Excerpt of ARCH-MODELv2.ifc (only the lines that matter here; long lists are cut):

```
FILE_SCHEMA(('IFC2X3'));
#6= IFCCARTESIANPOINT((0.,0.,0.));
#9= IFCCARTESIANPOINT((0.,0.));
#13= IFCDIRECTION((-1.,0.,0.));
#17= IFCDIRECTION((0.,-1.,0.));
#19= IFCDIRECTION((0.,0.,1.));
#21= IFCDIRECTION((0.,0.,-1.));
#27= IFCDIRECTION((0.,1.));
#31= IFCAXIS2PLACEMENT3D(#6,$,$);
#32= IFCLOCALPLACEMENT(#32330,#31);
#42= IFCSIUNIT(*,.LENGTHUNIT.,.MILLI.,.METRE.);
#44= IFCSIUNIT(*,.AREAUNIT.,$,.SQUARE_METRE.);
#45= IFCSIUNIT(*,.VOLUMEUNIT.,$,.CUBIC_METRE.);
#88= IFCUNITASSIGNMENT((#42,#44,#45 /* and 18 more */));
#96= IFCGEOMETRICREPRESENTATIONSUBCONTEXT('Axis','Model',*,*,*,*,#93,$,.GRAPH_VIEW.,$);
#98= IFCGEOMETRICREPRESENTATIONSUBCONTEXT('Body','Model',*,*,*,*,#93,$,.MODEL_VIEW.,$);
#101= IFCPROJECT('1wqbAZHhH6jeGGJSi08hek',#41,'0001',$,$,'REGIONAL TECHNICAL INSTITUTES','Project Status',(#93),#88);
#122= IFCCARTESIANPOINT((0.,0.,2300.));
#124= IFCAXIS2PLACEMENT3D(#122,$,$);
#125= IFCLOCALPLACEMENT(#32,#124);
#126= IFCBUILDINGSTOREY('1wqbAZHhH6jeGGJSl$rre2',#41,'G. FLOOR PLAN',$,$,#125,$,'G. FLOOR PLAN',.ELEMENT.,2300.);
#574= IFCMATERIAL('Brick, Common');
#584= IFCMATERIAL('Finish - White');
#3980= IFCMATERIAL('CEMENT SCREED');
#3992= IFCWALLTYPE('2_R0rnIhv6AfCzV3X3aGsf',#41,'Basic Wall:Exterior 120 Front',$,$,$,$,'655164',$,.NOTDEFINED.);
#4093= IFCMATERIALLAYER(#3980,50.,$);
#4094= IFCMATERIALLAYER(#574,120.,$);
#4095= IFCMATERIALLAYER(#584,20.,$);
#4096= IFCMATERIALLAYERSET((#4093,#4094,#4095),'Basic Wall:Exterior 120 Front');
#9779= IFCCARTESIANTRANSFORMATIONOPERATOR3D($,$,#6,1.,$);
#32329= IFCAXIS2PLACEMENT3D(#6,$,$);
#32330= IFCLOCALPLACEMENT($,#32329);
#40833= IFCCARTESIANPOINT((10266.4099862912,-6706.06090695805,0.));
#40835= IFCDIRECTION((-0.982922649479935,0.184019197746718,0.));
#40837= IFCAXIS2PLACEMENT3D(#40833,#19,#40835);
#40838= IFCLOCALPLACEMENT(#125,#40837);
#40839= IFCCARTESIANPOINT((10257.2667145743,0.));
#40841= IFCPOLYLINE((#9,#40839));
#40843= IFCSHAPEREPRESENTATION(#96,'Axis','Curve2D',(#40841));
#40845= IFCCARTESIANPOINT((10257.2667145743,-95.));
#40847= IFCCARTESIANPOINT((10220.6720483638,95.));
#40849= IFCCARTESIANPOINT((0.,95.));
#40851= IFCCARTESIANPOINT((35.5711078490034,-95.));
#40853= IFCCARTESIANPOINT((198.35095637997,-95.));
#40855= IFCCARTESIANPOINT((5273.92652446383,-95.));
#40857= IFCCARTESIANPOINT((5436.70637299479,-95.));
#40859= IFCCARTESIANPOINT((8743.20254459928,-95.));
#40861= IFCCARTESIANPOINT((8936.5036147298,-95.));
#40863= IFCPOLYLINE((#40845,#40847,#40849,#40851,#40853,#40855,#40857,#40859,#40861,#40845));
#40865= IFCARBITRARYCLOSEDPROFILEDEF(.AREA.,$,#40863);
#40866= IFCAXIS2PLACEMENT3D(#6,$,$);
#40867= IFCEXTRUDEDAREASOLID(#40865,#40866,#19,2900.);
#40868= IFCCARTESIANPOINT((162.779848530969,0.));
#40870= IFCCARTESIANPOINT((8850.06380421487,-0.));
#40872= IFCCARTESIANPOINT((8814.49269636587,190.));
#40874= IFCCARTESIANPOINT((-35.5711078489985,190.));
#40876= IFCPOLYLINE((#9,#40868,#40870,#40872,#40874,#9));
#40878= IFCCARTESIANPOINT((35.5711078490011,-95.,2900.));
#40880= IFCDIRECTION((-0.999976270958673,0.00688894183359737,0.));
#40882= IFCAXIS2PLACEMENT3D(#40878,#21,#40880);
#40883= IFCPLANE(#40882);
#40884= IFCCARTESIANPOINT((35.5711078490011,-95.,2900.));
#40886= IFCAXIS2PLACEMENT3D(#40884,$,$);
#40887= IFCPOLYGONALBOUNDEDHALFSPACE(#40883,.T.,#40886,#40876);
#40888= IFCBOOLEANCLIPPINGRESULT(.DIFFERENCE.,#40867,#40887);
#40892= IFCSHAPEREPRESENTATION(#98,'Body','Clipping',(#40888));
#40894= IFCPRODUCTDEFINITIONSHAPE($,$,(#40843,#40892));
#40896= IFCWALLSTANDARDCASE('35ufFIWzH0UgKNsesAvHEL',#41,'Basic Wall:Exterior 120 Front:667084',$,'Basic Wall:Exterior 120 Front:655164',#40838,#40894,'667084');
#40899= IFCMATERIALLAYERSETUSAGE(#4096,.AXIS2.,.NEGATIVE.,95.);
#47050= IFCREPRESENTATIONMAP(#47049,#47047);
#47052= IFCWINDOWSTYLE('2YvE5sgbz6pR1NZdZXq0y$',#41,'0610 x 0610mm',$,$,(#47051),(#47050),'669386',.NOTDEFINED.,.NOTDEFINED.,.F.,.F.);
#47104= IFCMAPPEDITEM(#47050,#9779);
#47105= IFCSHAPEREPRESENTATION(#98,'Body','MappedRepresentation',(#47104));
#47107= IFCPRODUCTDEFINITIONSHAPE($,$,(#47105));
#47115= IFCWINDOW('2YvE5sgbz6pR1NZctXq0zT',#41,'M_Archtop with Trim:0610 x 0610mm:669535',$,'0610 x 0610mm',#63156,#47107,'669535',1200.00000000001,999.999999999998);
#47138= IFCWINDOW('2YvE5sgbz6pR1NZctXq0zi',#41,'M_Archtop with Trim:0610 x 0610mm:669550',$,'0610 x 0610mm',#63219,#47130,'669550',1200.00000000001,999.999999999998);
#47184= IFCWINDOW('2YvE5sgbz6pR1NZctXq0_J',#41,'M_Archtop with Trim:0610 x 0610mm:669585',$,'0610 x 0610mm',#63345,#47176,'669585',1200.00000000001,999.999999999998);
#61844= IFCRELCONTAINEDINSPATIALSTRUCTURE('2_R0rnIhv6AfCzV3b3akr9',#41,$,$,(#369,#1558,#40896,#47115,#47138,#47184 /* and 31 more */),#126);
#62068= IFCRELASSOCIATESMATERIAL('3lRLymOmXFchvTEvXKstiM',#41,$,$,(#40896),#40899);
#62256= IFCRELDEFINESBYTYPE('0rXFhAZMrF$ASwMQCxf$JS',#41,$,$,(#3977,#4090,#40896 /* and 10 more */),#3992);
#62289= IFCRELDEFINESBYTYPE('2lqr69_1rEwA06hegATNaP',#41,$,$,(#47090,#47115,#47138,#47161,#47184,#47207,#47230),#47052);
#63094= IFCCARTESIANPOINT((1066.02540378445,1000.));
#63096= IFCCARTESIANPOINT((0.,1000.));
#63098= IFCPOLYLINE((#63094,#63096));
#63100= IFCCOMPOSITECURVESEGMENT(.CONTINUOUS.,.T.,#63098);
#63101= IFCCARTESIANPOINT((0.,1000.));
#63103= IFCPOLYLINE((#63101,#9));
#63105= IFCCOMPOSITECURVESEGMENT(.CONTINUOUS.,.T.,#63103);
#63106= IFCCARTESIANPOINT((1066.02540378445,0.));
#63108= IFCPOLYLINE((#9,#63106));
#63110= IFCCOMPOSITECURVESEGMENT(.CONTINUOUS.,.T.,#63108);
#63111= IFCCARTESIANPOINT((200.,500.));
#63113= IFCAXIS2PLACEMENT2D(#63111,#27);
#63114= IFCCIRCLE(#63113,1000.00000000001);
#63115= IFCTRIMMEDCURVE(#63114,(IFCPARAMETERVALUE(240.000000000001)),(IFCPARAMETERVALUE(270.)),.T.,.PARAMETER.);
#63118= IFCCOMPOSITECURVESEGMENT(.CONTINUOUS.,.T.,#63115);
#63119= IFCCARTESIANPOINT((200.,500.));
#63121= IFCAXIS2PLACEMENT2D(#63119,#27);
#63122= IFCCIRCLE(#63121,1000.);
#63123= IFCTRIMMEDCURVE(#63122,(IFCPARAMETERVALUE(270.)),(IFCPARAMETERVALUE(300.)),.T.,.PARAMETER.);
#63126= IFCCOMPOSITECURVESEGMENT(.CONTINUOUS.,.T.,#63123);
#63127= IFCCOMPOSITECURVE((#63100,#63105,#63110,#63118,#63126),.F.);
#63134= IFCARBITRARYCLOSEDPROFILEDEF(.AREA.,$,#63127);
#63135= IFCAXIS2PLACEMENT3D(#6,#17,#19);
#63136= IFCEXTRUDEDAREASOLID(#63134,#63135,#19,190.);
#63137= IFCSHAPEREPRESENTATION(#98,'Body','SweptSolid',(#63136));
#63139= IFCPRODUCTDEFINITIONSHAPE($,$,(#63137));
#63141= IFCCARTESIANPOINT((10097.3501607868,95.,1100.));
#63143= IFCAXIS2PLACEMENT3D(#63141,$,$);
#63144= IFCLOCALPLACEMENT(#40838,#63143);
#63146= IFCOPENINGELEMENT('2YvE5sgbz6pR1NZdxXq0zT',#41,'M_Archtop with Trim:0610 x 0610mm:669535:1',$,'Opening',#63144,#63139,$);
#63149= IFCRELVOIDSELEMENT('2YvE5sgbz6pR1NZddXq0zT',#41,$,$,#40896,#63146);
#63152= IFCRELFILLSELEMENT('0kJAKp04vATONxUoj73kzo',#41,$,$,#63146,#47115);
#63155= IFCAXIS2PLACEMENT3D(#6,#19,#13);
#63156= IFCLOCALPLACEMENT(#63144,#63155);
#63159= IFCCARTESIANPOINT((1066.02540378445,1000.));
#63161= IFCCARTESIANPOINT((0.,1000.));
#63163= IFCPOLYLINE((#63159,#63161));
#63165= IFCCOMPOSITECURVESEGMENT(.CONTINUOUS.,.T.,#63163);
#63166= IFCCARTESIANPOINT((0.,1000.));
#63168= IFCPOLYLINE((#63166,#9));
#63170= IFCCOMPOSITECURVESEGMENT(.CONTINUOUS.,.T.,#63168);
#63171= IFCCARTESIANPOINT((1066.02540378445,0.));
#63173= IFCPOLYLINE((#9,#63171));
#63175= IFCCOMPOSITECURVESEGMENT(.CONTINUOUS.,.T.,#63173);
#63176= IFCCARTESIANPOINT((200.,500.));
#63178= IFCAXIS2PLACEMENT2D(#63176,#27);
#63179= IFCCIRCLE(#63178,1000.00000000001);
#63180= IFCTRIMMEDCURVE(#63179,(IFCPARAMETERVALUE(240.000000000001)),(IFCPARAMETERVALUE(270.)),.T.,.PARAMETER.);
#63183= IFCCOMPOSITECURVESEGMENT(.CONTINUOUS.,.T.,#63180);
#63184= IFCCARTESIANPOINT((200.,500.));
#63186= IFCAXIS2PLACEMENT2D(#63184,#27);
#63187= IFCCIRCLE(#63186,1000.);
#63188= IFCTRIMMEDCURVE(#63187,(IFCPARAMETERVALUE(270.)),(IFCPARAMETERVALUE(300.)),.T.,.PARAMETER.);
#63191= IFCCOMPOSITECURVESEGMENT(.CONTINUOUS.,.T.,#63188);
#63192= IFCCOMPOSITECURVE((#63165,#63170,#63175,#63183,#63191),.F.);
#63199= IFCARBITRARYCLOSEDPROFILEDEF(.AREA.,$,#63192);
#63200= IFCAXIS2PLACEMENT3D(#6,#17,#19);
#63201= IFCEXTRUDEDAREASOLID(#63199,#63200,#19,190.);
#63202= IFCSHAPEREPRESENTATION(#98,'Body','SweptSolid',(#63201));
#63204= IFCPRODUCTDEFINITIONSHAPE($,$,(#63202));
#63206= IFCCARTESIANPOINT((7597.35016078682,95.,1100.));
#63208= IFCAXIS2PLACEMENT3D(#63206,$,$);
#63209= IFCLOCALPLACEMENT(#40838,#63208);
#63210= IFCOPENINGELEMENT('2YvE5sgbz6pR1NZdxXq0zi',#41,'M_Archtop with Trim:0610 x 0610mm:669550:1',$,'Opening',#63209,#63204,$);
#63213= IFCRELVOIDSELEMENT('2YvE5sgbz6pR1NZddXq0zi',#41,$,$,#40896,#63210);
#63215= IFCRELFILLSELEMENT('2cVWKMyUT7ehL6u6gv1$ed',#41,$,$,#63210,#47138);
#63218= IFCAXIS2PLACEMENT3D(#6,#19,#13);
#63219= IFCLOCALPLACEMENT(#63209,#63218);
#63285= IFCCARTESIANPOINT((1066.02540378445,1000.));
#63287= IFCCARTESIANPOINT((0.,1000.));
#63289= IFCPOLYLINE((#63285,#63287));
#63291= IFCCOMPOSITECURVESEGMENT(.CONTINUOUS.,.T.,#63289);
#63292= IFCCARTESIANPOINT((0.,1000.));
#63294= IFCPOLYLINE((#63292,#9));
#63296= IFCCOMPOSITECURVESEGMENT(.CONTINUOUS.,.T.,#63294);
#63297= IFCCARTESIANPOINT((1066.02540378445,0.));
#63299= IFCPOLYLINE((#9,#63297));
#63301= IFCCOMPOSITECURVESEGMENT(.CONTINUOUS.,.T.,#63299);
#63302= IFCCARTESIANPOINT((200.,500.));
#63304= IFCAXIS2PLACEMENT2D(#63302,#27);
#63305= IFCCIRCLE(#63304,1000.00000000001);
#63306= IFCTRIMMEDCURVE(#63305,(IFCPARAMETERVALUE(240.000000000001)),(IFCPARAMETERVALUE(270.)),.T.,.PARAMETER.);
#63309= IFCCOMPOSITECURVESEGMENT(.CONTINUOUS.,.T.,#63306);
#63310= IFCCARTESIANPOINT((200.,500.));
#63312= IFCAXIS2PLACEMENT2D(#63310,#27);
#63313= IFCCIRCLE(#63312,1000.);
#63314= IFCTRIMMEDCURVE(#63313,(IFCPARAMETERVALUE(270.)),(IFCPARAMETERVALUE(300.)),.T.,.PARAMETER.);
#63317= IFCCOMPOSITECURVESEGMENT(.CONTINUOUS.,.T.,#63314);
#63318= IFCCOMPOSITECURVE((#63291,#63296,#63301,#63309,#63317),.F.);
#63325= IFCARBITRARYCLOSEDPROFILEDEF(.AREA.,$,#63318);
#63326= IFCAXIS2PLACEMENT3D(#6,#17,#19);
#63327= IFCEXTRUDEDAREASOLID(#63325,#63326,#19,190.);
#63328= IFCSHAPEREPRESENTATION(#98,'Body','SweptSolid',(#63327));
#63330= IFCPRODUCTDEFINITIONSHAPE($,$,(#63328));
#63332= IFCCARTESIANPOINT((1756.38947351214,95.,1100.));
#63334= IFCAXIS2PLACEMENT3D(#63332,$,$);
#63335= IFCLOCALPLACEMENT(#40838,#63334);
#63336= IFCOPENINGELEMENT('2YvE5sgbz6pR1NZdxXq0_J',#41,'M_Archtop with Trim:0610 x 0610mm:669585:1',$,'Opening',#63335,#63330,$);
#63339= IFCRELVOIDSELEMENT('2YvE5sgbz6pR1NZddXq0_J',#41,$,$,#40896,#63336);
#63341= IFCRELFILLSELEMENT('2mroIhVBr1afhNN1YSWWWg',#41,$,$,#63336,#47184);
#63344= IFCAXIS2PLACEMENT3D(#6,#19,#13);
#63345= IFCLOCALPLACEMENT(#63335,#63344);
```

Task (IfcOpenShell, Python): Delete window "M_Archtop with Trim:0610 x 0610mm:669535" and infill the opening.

```python
import ifcopenshell
import ifcopenshell.api.feature
import ifcopenshell.api.root
import ifcopenshell.geom
import ifcopenshell.util.shape

model = ifcopenshell.open("ARCH-MODELv2.ifc")
settings = ifcopenshell.geom.settings()


def volume(element):
    """Net volume in cubic metres, openings subtracted."""
    shape = ifcopenshell.geom.create_shape(settings, element)
    return ifcopenshell.util.shape.get_volume(shape.geometry)


window = model.by_id(47115)
opening = window.FillsVoids[0].RelatingOpeningElement
wall = opening.VoidsElements[0].RelatingBuildingElement
before = volume(wall)

ifcopenshell.api.root.remove_product(model, product=window)
ifcopenshell.api.feature.remove_feature(model, feature=opening)

after = volume(wall)

print(f"wall volume {before:.3f} -> {after:.3f} m3")

model.write("ARCH-MODELv2_edited.ifc")
```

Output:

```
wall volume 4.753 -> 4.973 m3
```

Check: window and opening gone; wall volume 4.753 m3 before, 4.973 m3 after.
